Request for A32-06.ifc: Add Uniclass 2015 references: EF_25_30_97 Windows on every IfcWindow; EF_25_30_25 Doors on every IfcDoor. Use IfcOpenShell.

First a look at what the model holds.

```python
import ifcopenshell

model = ifcopenshell.open("A32-06.ifc")
print(model.schema)
print("classifications:", [c.Name for c in model.by_type("IfcClassification")])
for ifc_class in ("IfcDoor", "IfcRoof", "IfcStair", "IfcWall", "IfcWindow"):
    print(ifc_class, len(model.by_type(ifc_class)))
```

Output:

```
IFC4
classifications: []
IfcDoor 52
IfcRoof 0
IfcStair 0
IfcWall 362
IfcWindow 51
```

```python
import ifcopenshell
import ifcopenshell.api.classification

model = ifcopenshell.open("A32-06.ifc")

system = ifcopenshell.api.classification.add_classification(model, classification="Uniclass 2015")

codes = {
    "IfcWindow": ("EF_25_30_97", "Windows"),
    "IfcDoor": ("EF_25_30_25", "Doors"),
}
for ifc_class, (code, name) in codes.items():
    products = model.by_type(ifc_class)
    ifcopenshell.api.classification.add_reference(
        model, products=products, classification=system, identification=code, name=name
    )
    print(code, len(products))

model.write("A32-06_edited.ifc")
```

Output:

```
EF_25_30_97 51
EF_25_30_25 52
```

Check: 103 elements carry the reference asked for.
